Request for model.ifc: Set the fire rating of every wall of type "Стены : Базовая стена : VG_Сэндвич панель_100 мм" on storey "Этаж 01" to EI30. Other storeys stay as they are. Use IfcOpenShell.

First a look at what the model holds.

```python
import ifcopenshell
import ifcopenshell.util.element

model = ifcopenshell.open("model.ifc")
print(model.schema)
storey = next(s for s in model.by_type("IfcBuildingStorey") if s.Name == "Этаж 01")
walls = [e for e in ifcopenshell.util.element.get_decomposition(storey) if e.is_a("IfcWall")]
seen = {}
for e in walls:
    element_type = ifcopenshell.util.element.get_type(e)
    key = (element_type.Name if element_type != e and element_type else None, ifcopenshell.util.element.get_pset(e, "Pset_WallCommon", "FireRating"))
    seen[key] = seen.get(key, 0) + 1
for (name, value), count in sorted(seen.items(), key=str):
    print(count, "x", name, "|", value)
```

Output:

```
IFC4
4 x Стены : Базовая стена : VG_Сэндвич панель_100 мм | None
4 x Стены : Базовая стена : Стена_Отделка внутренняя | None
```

```python
import ifcopenshell
import ifcopenshell.api.pset
import ifcopenshell.util.element

model = ifcopenshell.open("model.ifc")

storey = next(s for s in model.by_type("IfcBuildingStorey") if s.Name == "Этаж 01")
walls = [e for e in ifcopenshell.util.element.get_decomposition(storey) if e.is_a("IfcWall")]

count = 0
for e in walls:
    element_type = ifcopenshell.util.element.get_type(e)
    if element_type in (None, e) or element_type.Name != "Стены : Базовая стена : VG_Сэндвич панель_100 мм":
        continue
    # add_pset returns the element's existing set when there is one.
    pset = ifcopenshell.api.pset.add_pset(model, product=e, name="Pset_WallCommon")
    ifcopenshell.api.pset.edit_pset(model, pset=pset, properties={"FireRating": "EI30"})
    count += 1

print(count, "walls updated")

model.write("model_v2.ifc")
```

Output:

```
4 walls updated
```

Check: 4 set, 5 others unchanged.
